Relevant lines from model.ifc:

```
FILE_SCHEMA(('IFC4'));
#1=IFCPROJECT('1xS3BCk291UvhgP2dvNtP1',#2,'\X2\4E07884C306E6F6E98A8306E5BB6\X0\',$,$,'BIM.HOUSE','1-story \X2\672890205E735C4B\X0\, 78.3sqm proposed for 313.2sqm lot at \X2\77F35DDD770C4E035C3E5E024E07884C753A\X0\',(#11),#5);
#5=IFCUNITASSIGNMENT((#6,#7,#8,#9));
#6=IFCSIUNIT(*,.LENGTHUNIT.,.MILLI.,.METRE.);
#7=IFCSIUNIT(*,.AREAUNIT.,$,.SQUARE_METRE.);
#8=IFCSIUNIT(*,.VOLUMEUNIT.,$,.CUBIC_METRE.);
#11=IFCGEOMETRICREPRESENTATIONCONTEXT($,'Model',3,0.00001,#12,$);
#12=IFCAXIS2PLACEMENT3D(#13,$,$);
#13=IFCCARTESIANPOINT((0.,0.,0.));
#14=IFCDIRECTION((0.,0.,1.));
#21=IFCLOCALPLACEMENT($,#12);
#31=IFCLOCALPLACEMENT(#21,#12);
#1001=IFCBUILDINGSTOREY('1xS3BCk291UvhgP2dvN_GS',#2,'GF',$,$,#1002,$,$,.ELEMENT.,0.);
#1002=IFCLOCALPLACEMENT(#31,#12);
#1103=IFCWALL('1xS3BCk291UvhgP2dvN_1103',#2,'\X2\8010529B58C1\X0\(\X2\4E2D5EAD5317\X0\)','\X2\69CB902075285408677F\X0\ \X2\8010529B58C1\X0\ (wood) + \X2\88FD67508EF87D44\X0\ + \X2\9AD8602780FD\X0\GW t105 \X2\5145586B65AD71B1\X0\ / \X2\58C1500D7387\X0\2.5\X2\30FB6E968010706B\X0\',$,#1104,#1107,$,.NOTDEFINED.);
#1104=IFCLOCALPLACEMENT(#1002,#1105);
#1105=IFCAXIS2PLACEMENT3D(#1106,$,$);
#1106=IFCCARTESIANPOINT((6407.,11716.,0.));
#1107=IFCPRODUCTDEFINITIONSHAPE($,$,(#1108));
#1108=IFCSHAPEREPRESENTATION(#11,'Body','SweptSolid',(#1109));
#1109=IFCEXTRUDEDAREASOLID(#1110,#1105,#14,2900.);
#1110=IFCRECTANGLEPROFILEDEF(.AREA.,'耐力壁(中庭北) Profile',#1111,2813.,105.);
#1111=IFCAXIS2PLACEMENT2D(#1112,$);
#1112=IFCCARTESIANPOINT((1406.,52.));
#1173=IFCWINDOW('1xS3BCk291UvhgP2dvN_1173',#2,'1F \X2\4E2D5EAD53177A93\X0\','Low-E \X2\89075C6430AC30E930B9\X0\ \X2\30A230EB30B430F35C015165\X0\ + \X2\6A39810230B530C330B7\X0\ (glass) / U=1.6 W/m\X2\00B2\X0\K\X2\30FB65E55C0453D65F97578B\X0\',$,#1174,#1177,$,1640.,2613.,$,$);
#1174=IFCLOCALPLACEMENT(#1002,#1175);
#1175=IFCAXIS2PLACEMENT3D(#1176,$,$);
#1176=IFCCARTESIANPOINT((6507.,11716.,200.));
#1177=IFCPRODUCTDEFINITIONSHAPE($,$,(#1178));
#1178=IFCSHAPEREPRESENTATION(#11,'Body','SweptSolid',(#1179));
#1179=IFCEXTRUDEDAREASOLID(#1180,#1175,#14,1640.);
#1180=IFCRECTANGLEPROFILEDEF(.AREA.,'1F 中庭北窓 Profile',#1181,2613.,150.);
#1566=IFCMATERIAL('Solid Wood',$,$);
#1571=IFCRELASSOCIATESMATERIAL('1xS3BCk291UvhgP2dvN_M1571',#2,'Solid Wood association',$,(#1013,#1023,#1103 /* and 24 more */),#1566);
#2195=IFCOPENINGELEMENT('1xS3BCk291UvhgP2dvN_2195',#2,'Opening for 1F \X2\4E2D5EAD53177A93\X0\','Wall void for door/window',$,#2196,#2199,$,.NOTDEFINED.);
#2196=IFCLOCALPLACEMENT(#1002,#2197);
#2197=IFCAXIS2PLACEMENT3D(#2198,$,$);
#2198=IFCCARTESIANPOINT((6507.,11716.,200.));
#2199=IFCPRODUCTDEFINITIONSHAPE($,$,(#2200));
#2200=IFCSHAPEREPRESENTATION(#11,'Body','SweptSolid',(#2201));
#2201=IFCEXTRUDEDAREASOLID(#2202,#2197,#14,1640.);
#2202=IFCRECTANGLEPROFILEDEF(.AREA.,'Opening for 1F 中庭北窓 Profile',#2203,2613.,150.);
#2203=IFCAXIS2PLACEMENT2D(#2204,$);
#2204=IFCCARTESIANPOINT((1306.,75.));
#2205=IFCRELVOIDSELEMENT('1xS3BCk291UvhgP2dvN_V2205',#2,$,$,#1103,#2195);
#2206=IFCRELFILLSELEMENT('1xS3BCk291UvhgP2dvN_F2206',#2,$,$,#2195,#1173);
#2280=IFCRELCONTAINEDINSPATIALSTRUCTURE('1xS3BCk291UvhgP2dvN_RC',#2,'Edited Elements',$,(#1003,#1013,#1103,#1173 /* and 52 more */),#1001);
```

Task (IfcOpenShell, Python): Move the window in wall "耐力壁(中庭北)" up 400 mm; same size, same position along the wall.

```python
import numpy as np
import ifcopenshell
import ifcopenshell.api.geometry
import ifcopenshell.util.placement
import ifcopenshell.util.unit

model = ifcopenshell.open("model.ifc")
unit_scale = ifcopenshell.util.unit.calculate_unit_scale(model)

window = model.by_guid("1xS3BCk291UvhgP2dvN_1173")
opening = window.FillsVoids[0].RelatingOpeningElement
dz = 400.0

shift = np.array([0.0, 0.0, dz])
# The window is not placed relative to its opening, so move both.
for product in (opening, window):
    matrix = ifcopenshell.util.placement.get_local_placement(product.ObjectPlacement)
    matrix[:3, 3] += shift
    ifcopenshell.api.geometry.edit_object_placement(model, product=product, matrix=matrix, is_si=False)

print(f"moved by {dz * unit_scale:+.3f} m")

model.write("model_edited.ifc")
```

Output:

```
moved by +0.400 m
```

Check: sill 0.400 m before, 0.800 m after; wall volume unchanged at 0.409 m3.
